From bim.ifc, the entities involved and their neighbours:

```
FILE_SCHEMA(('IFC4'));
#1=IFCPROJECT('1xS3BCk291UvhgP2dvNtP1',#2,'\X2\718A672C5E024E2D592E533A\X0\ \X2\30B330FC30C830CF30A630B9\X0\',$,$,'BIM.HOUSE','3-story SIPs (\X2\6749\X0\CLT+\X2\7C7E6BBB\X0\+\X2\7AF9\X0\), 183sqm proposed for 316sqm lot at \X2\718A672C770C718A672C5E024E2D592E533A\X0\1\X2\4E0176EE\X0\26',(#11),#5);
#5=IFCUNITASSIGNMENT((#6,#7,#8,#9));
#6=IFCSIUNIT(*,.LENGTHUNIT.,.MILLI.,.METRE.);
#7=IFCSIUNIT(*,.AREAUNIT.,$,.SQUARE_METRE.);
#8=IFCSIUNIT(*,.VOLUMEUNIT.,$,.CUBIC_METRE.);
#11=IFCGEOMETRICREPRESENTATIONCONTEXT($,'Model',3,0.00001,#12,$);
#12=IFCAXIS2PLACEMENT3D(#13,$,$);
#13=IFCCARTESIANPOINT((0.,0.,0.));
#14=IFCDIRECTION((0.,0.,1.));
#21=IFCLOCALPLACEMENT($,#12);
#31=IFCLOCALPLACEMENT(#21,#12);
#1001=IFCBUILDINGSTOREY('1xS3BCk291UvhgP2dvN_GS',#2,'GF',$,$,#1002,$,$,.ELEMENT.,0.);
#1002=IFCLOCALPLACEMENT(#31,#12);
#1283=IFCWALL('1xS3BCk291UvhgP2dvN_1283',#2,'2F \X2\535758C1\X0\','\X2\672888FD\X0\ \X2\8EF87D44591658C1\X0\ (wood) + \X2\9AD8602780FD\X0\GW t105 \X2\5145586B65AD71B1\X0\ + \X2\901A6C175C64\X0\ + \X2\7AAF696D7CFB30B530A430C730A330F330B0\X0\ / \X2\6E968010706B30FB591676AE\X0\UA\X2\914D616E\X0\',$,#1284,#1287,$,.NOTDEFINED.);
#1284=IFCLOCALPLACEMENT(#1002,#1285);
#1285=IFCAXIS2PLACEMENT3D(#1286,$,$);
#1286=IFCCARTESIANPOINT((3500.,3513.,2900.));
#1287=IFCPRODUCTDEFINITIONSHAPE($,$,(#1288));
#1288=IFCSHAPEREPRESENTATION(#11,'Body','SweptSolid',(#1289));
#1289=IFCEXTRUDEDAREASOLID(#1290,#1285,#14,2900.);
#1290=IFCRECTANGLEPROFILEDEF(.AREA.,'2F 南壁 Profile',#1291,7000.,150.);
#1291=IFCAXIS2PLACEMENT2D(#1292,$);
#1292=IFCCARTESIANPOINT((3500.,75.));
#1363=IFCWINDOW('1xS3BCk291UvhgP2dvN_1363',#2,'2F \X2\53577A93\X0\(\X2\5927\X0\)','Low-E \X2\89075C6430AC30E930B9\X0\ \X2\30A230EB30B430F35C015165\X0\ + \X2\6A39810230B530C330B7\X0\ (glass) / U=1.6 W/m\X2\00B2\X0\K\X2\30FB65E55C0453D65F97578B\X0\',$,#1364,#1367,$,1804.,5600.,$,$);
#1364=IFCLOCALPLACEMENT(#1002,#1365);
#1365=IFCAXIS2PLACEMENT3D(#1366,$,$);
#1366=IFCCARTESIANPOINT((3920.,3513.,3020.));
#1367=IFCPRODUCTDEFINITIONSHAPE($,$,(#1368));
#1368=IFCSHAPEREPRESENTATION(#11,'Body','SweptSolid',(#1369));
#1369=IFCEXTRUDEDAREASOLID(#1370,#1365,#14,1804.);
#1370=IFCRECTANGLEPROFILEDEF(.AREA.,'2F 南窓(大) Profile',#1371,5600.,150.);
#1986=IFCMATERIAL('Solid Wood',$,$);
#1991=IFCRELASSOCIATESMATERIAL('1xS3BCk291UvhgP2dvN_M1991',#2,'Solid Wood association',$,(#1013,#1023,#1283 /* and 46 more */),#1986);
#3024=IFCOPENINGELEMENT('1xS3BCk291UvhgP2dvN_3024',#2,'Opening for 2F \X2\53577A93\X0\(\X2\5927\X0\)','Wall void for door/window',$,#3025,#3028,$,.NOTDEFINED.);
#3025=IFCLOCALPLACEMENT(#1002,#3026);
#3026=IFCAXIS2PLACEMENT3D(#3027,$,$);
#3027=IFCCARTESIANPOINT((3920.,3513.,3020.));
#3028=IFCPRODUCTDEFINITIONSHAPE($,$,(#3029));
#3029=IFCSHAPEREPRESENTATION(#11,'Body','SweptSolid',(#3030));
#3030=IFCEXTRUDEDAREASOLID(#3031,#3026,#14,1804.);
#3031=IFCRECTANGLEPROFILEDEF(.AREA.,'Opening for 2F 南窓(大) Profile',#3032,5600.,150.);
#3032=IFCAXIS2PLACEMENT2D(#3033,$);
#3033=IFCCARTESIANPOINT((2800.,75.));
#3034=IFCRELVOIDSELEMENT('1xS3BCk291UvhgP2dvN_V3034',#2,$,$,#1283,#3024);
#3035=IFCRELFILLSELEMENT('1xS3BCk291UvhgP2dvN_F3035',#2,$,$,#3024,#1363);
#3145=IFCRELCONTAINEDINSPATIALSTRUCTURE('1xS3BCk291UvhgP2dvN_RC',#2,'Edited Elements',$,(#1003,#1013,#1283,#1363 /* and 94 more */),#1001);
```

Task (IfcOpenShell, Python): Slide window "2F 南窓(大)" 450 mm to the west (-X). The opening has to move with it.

```python
import ifcopenshell
import ifcopenshell.api.geometry
import ifcopenshell.util.placement
import ifcopenshell.util.unit

model = ifcopenshell.open("bim.ifc")
unit_scale = ifcopenshell.util.unit.calculate_unit_scale(model)

window = model.by_guid("1xS3BCk291UvhgP2dvN_1363")
opening = window.FillsVoids[0].RelatingOpeningElement
wall = opening.VoidsElements[0].RelatingBuildingElement

wall_matrix = ifcopenshell.util.placement.get_local_placement(wall.ObjectPlacement)
shift = wall_matrix[:3, 0] * -0.45 / unit_scale
before = ifcopenshell.util.placement.get_local_placement(window.ObjectPlacement)[:3, 3].copy()

# The window is not placed relative to its opening, so move both.
for product in (opening, window):
    matrix = ifcopenshell.util.placement.get_local_placement(product.ObjectPlacement)
    matrix[:3, 3] += shift
    ifcopenshell.api.geometry.edit_object_placement(model, product=product, matrix=matrix, is_si=False)

after = ifcopenshell.util.placement.get_local_placement(window.ObjectPlacement)[:3, 3]
print("window moved by", (after - before).round(3) + 0.0)

model.write("bim_rev.ifc")
```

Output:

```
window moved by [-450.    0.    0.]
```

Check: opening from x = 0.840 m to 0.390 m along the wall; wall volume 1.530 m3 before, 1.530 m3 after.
